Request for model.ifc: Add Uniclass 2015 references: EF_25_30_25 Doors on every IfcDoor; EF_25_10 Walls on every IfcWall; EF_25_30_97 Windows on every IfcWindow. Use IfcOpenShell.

First a look at what the model holds.

```python
import ifcopenshell

model = ifcopenshell.open("model.ifc")
print(model.schema)
print("classifications:", [c.Name for c in model.by_type("IfcClassification")])
for ifc_class in ("IfcDoor", "IfcRoof", "IfcStair", "IfcWall", "IfcWindow"):
    print(ifc_class, len(model.by_type(ifc_class)))
```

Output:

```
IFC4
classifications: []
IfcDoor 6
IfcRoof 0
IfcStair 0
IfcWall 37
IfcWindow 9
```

```python
import ifcopenshell
import ifcopenshell.api.classification

model = ifcopenshell.open("model.ifc")

system = ifcopenshell.api.classification.add_classification(model, classification="Uniclass 2015")

codes = {
    "IfcDoor": ("EF_25_30_25", "Doors"),
    "IfcWall": ("EF_25_10", "Walls"),
    "IfcWindow": ("EF_25_30_97", "Windows"),
}
for ifc_class, (code, name) in codes.items():
    products = model.by_type(ifc_class)
    ifcopenshell.api.classification.add_reference(
        model, products=products, classification=system, identification=code, name=name
    )
    print(code, len(products))

model.write("model-out.ifc")
```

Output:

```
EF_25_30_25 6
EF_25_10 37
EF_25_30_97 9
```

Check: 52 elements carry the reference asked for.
